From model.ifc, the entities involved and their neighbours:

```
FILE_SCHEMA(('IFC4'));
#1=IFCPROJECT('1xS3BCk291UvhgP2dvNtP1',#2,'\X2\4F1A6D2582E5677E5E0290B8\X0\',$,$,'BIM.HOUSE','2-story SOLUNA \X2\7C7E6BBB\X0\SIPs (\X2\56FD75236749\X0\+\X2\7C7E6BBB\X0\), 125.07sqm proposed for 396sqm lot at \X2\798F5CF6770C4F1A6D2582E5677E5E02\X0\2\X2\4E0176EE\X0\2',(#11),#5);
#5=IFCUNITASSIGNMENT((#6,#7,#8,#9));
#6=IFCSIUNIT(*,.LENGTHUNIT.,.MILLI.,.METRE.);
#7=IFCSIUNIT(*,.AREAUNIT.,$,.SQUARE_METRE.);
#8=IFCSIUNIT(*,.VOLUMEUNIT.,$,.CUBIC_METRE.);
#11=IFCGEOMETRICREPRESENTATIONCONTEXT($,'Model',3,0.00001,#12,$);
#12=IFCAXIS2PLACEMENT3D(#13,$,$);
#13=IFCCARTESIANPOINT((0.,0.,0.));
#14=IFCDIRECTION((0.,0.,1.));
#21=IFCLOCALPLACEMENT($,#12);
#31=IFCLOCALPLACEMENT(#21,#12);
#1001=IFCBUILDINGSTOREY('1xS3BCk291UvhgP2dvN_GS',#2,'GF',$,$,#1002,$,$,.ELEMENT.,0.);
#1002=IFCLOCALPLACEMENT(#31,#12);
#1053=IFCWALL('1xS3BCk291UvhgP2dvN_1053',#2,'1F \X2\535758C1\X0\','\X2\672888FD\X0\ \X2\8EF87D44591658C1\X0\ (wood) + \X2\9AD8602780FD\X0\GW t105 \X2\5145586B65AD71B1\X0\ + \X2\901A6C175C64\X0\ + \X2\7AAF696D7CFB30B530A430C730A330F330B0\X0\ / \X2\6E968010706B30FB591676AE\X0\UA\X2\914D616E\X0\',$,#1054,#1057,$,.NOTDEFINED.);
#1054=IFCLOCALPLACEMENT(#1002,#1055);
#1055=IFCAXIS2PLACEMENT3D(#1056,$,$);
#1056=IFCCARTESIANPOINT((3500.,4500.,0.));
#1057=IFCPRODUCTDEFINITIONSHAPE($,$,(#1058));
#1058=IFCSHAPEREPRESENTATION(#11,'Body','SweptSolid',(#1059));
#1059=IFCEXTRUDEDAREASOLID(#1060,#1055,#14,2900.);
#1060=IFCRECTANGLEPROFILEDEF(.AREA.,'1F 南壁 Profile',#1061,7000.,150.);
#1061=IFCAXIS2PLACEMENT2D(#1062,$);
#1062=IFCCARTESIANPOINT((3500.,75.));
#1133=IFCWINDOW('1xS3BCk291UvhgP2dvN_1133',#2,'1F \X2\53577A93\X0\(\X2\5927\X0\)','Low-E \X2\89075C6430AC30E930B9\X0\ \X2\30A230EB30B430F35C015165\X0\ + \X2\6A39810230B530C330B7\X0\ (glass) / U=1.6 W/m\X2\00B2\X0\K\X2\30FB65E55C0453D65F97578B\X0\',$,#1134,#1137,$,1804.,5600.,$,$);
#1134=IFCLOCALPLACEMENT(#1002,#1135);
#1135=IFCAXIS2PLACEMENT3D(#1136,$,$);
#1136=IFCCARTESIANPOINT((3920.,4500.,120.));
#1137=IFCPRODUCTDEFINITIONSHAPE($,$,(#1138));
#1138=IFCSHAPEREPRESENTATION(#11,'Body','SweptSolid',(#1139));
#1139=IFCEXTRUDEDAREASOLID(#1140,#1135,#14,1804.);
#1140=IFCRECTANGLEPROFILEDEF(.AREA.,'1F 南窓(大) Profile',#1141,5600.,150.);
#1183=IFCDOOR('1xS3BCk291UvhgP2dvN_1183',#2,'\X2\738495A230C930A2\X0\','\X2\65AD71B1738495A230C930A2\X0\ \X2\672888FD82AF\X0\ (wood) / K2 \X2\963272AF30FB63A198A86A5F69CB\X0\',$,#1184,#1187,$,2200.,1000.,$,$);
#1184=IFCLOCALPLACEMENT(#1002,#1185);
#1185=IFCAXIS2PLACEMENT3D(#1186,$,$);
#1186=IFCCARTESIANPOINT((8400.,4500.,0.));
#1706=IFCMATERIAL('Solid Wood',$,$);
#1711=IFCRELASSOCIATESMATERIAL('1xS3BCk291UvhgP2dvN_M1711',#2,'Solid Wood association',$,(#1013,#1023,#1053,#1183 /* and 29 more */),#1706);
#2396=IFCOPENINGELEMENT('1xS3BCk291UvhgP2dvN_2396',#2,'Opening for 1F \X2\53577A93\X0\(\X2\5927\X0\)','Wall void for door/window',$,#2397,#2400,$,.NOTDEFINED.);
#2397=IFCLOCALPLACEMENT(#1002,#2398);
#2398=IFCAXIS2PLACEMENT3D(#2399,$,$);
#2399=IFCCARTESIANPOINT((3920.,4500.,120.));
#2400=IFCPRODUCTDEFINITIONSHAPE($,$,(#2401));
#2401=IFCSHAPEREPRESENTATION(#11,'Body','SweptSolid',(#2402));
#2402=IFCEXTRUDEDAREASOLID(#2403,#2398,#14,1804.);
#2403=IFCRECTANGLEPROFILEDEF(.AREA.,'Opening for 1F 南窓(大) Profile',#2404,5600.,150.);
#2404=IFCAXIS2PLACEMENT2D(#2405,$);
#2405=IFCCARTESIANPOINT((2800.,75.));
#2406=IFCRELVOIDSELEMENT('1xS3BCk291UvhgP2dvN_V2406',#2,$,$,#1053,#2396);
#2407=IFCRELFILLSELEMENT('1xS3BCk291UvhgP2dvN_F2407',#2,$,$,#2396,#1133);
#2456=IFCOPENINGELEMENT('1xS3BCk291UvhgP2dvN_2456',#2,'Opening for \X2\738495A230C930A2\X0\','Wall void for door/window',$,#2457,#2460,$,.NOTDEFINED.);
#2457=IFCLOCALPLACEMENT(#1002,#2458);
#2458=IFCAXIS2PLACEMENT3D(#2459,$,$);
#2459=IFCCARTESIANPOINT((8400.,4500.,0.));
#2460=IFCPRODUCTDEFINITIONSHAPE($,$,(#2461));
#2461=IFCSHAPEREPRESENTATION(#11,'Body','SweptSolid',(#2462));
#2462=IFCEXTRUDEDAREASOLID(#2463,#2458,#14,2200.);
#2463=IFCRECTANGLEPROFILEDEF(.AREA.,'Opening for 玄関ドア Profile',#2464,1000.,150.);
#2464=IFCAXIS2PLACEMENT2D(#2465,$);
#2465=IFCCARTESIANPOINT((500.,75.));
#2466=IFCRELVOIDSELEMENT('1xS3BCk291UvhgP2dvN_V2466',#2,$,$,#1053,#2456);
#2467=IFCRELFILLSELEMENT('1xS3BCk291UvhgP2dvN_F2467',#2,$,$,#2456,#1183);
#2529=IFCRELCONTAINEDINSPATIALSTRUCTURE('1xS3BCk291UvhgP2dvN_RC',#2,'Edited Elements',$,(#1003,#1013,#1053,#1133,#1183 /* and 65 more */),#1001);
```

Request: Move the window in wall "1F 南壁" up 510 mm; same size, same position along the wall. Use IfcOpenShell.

```python
import numpy as np
import ifcopenshell
import ifcopenshell.api.geometry
import ifcopenshell.util.placement
import ifcopenshell.util.unit

model = ifcopenshell.open("model.ifc")
unit_scale = ifcopenshell.util.unit.calculate_unit_scale(model)

window = model.by_id(1133)
opening = window.FillsVoids[0].RelatingOpeningElement
dz = 510.0

shift = np.array([0.0, 0.0, dz])
# The window is not placed relative to its opening, so move both.
for product in (opening, window):
    matrix = ifcopenshell.util.placement.get_local_placement(product.ObjectPlacement)
    matrix[:3, 3] += shift
    ifcopenshell.api.geometry.edit_object_placement(model, product=product, matrix=matrix, is_si=False)

print(f"moved by {dz * unit_scale:+.3f} m")

model.write("model_v2.ifc")
```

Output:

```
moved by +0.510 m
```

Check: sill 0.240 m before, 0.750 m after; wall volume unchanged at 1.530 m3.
